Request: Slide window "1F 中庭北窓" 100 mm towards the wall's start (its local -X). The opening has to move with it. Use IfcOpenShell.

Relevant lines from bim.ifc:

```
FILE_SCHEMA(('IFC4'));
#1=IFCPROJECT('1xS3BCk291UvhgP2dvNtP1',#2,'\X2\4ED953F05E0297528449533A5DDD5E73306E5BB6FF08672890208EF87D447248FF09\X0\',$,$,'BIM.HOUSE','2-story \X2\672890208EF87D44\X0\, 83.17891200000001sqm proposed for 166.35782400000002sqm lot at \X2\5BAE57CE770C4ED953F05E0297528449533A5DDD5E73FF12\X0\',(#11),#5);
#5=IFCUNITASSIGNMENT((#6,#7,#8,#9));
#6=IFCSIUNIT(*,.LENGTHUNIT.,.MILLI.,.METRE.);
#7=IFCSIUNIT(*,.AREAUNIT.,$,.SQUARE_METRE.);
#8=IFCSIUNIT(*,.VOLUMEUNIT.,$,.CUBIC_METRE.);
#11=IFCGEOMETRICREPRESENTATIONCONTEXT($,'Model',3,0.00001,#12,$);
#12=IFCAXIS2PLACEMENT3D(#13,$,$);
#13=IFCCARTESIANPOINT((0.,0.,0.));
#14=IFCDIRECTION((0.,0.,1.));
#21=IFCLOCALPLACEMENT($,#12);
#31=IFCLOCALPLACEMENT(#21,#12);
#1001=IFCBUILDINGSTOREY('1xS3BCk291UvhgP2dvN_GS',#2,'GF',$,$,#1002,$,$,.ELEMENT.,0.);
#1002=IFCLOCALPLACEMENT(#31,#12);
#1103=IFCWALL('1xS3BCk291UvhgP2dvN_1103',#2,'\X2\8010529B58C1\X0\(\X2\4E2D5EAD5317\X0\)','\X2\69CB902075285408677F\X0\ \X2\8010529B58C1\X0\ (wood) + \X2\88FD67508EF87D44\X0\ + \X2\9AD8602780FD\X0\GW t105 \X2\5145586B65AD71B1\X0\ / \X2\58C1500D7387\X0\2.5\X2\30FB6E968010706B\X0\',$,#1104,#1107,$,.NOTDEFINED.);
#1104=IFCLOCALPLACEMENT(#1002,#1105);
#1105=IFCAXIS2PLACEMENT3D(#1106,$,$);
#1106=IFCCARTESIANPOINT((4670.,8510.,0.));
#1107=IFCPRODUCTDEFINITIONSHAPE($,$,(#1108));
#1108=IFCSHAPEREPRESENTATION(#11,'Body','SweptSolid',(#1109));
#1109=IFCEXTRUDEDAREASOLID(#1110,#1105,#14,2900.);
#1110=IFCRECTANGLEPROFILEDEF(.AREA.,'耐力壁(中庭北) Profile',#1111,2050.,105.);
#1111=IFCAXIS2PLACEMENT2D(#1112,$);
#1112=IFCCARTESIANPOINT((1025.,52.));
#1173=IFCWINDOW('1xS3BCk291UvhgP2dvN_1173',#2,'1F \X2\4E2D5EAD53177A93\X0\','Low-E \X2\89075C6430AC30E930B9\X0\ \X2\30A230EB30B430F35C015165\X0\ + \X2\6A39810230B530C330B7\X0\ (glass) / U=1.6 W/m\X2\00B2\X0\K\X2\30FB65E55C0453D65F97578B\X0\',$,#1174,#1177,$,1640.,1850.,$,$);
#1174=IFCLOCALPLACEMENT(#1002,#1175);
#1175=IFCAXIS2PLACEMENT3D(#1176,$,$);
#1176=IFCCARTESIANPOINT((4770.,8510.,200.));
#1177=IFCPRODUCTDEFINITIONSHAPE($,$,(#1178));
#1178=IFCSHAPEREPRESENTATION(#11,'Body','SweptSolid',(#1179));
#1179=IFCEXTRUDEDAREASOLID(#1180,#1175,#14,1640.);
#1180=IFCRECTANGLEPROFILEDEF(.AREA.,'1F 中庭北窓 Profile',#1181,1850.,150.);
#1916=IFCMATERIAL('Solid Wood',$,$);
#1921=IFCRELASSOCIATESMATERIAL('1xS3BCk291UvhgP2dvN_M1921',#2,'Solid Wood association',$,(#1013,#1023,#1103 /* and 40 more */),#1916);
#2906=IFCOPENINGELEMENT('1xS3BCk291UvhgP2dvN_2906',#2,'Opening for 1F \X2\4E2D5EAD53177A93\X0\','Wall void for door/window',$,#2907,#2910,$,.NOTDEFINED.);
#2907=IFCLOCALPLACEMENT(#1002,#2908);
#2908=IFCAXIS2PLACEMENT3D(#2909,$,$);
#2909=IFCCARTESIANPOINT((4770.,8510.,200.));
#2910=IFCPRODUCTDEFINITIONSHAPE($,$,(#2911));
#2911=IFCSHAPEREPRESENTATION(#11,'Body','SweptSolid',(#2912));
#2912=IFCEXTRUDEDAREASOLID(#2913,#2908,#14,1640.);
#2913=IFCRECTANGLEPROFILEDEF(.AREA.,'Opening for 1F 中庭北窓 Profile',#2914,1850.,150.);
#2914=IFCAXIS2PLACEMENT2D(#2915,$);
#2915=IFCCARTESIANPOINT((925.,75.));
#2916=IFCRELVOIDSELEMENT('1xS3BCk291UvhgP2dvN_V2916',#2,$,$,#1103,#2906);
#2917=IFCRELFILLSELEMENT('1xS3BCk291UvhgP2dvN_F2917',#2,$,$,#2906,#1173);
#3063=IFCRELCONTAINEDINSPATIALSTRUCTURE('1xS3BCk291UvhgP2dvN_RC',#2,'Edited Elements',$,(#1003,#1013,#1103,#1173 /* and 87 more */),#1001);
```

```python
import ifcopenshell
import ifcopenshell.api.geometry
import ifcopenshell.util.placement

model = ifcopenshell.open("bim.ifc")

window = model.by_id(1173)
opening = window.FillsVoids[0].RelatingOpeningElement
wall = opening.VoidsElements[0].RelatingBuildingElement

wall_matrix = ifcopenshell.util.placement.get_local_placement(wall.ObjectPlacement)
shift = wall_matrix[:3, 0] * -100.0
before = ifcopenshell.util.placement.get_local_placement(window.ObjectPlacement)[:3, 3].copy()

# The window is not placed relative to its opening, so move both.
for product in (opening, window):
    matrix = ifcopenshell.util.placement.get_local_placement(product.ObjectPlacement)
    matrix[:3, 3] += shift
    ifcopenshell.api.geometry.edit_object_placement(model, product=product, matrix=matrix, is_si=False)

after = ifcopenshell.util.placement.get_local_placement(window.ObjectPlacement)[:3, 3]
print("window moved by", (after - before).round(3) + 0.0)

model.write("bim_v2.ifc")
```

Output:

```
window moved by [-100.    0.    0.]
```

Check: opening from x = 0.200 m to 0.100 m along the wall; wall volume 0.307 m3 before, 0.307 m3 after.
